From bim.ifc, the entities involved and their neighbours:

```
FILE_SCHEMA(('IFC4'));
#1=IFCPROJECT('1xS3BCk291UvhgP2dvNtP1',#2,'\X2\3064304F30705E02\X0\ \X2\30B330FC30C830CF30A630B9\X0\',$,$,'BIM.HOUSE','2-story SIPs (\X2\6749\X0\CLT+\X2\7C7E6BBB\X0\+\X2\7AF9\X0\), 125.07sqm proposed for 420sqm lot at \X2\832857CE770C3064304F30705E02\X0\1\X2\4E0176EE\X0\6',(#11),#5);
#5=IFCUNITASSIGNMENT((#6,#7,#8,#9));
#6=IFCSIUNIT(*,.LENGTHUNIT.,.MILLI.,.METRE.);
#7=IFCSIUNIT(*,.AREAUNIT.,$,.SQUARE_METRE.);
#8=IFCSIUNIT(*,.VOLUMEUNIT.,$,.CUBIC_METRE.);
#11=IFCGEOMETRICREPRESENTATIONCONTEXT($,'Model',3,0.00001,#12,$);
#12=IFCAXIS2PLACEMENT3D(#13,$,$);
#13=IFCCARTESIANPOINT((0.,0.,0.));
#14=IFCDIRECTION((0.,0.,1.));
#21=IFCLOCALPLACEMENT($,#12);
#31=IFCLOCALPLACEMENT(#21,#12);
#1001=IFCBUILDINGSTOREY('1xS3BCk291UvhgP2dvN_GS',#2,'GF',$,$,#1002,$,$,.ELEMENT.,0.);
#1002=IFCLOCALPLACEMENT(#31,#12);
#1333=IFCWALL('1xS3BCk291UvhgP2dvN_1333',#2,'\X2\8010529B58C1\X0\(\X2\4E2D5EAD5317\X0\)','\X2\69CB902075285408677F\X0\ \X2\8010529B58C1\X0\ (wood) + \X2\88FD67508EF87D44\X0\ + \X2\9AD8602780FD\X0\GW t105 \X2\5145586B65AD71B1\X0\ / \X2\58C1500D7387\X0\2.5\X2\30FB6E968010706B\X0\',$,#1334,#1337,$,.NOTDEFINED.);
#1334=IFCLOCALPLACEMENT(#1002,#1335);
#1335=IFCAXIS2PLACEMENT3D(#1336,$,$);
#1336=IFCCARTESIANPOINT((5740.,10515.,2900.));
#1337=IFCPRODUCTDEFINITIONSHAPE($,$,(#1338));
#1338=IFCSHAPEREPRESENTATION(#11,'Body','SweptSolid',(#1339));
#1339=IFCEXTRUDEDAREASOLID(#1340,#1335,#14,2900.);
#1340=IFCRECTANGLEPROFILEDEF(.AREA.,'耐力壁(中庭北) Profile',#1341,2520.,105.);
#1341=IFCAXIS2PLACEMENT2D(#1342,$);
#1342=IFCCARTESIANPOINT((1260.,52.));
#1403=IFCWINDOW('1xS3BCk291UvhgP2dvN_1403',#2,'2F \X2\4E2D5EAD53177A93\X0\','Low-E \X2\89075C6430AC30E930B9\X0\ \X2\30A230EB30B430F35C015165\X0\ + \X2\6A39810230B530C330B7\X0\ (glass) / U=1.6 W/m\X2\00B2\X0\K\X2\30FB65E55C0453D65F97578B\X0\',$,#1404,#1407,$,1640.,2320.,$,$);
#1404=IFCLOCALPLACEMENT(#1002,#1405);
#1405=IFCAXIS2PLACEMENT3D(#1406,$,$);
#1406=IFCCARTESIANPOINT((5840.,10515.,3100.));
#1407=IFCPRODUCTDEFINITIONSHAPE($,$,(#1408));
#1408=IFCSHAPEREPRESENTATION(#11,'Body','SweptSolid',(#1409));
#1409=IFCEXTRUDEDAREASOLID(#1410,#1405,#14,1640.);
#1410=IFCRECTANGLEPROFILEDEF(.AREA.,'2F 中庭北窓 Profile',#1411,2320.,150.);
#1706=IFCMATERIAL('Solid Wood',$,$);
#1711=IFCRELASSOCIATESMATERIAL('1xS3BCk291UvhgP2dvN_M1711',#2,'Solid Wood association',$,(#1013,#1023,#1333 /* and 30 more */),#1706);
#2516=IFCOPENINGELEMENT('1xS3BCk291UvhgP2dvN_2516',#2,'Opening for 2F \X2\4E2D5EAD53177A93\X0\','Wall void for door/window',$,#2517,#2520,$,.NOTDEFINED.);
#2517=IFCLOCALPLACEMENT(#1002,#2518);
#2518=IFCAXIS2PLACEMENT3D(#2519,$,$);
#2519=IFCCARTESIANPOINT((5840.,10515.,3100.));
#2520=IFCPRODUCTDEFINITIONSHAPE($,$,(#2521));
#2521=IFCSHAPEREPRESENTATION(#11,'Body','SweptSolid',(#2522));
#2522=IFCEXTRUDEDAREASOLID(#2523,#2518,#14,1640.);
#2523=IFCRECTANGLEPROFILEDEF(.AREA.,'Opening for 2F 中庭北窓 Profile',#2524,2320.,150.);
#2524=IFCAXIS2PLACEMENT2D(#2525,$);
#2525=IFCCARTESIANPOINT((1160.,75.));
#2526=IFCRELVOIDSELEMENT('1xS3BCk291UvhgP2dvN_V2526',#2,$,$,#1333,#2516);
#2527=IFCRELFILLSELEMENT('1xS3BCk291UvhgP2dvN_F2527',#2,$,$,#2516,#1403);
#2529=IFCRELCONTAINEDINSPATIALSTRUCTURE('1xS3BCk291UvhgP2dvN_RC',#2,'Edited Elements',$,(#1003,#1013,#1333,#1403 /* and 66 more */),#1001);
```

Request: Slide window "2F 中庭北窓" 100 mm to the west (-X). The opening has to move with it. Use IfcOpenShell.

```python
import ifcopenshell
import ifcopenshell.api.geometry
import ifcopenshell.util.placement

model = ifcopenshell.open("bim.ifc")

window = model.by_id(1403)
opening = window.FillsVoids[0].RelatingOpeningElement
wall = opening.VoidsElements[0].RelatingBuildingElement

wall_matrix = ifcopenshell.util.placement.get_local_placement(wall.ObjectPlacement)
shift = wall_matrix[:3, 0] * -100.0
before = ifcopenshell.util.placement.get_local_placement(window.ObjectPlacement)[:3, 3].copy()

# The window is not placed relative to its opening, so move both.
for product in (opening, window):
    matrix = ifcopenshell.util.placement.get_local_placement(product.ObjectPlacement)
    matrix[:3, 3] += shift
    ifcopenshell.api.geometry.edit_object_placement(model, product=product, matrix=matrix, is_si=False)

after = ifcopenshell.util.placement.get_local_placement(window.ObjectPlacement)[:3, 3]
print("window moved by", (after - before).round(3) + 0.0)

model.write("bim_updated.ifc")
```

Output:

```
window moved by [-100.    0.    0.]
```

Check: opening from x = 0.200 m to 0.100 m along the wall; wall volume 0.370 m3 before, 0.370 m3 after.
